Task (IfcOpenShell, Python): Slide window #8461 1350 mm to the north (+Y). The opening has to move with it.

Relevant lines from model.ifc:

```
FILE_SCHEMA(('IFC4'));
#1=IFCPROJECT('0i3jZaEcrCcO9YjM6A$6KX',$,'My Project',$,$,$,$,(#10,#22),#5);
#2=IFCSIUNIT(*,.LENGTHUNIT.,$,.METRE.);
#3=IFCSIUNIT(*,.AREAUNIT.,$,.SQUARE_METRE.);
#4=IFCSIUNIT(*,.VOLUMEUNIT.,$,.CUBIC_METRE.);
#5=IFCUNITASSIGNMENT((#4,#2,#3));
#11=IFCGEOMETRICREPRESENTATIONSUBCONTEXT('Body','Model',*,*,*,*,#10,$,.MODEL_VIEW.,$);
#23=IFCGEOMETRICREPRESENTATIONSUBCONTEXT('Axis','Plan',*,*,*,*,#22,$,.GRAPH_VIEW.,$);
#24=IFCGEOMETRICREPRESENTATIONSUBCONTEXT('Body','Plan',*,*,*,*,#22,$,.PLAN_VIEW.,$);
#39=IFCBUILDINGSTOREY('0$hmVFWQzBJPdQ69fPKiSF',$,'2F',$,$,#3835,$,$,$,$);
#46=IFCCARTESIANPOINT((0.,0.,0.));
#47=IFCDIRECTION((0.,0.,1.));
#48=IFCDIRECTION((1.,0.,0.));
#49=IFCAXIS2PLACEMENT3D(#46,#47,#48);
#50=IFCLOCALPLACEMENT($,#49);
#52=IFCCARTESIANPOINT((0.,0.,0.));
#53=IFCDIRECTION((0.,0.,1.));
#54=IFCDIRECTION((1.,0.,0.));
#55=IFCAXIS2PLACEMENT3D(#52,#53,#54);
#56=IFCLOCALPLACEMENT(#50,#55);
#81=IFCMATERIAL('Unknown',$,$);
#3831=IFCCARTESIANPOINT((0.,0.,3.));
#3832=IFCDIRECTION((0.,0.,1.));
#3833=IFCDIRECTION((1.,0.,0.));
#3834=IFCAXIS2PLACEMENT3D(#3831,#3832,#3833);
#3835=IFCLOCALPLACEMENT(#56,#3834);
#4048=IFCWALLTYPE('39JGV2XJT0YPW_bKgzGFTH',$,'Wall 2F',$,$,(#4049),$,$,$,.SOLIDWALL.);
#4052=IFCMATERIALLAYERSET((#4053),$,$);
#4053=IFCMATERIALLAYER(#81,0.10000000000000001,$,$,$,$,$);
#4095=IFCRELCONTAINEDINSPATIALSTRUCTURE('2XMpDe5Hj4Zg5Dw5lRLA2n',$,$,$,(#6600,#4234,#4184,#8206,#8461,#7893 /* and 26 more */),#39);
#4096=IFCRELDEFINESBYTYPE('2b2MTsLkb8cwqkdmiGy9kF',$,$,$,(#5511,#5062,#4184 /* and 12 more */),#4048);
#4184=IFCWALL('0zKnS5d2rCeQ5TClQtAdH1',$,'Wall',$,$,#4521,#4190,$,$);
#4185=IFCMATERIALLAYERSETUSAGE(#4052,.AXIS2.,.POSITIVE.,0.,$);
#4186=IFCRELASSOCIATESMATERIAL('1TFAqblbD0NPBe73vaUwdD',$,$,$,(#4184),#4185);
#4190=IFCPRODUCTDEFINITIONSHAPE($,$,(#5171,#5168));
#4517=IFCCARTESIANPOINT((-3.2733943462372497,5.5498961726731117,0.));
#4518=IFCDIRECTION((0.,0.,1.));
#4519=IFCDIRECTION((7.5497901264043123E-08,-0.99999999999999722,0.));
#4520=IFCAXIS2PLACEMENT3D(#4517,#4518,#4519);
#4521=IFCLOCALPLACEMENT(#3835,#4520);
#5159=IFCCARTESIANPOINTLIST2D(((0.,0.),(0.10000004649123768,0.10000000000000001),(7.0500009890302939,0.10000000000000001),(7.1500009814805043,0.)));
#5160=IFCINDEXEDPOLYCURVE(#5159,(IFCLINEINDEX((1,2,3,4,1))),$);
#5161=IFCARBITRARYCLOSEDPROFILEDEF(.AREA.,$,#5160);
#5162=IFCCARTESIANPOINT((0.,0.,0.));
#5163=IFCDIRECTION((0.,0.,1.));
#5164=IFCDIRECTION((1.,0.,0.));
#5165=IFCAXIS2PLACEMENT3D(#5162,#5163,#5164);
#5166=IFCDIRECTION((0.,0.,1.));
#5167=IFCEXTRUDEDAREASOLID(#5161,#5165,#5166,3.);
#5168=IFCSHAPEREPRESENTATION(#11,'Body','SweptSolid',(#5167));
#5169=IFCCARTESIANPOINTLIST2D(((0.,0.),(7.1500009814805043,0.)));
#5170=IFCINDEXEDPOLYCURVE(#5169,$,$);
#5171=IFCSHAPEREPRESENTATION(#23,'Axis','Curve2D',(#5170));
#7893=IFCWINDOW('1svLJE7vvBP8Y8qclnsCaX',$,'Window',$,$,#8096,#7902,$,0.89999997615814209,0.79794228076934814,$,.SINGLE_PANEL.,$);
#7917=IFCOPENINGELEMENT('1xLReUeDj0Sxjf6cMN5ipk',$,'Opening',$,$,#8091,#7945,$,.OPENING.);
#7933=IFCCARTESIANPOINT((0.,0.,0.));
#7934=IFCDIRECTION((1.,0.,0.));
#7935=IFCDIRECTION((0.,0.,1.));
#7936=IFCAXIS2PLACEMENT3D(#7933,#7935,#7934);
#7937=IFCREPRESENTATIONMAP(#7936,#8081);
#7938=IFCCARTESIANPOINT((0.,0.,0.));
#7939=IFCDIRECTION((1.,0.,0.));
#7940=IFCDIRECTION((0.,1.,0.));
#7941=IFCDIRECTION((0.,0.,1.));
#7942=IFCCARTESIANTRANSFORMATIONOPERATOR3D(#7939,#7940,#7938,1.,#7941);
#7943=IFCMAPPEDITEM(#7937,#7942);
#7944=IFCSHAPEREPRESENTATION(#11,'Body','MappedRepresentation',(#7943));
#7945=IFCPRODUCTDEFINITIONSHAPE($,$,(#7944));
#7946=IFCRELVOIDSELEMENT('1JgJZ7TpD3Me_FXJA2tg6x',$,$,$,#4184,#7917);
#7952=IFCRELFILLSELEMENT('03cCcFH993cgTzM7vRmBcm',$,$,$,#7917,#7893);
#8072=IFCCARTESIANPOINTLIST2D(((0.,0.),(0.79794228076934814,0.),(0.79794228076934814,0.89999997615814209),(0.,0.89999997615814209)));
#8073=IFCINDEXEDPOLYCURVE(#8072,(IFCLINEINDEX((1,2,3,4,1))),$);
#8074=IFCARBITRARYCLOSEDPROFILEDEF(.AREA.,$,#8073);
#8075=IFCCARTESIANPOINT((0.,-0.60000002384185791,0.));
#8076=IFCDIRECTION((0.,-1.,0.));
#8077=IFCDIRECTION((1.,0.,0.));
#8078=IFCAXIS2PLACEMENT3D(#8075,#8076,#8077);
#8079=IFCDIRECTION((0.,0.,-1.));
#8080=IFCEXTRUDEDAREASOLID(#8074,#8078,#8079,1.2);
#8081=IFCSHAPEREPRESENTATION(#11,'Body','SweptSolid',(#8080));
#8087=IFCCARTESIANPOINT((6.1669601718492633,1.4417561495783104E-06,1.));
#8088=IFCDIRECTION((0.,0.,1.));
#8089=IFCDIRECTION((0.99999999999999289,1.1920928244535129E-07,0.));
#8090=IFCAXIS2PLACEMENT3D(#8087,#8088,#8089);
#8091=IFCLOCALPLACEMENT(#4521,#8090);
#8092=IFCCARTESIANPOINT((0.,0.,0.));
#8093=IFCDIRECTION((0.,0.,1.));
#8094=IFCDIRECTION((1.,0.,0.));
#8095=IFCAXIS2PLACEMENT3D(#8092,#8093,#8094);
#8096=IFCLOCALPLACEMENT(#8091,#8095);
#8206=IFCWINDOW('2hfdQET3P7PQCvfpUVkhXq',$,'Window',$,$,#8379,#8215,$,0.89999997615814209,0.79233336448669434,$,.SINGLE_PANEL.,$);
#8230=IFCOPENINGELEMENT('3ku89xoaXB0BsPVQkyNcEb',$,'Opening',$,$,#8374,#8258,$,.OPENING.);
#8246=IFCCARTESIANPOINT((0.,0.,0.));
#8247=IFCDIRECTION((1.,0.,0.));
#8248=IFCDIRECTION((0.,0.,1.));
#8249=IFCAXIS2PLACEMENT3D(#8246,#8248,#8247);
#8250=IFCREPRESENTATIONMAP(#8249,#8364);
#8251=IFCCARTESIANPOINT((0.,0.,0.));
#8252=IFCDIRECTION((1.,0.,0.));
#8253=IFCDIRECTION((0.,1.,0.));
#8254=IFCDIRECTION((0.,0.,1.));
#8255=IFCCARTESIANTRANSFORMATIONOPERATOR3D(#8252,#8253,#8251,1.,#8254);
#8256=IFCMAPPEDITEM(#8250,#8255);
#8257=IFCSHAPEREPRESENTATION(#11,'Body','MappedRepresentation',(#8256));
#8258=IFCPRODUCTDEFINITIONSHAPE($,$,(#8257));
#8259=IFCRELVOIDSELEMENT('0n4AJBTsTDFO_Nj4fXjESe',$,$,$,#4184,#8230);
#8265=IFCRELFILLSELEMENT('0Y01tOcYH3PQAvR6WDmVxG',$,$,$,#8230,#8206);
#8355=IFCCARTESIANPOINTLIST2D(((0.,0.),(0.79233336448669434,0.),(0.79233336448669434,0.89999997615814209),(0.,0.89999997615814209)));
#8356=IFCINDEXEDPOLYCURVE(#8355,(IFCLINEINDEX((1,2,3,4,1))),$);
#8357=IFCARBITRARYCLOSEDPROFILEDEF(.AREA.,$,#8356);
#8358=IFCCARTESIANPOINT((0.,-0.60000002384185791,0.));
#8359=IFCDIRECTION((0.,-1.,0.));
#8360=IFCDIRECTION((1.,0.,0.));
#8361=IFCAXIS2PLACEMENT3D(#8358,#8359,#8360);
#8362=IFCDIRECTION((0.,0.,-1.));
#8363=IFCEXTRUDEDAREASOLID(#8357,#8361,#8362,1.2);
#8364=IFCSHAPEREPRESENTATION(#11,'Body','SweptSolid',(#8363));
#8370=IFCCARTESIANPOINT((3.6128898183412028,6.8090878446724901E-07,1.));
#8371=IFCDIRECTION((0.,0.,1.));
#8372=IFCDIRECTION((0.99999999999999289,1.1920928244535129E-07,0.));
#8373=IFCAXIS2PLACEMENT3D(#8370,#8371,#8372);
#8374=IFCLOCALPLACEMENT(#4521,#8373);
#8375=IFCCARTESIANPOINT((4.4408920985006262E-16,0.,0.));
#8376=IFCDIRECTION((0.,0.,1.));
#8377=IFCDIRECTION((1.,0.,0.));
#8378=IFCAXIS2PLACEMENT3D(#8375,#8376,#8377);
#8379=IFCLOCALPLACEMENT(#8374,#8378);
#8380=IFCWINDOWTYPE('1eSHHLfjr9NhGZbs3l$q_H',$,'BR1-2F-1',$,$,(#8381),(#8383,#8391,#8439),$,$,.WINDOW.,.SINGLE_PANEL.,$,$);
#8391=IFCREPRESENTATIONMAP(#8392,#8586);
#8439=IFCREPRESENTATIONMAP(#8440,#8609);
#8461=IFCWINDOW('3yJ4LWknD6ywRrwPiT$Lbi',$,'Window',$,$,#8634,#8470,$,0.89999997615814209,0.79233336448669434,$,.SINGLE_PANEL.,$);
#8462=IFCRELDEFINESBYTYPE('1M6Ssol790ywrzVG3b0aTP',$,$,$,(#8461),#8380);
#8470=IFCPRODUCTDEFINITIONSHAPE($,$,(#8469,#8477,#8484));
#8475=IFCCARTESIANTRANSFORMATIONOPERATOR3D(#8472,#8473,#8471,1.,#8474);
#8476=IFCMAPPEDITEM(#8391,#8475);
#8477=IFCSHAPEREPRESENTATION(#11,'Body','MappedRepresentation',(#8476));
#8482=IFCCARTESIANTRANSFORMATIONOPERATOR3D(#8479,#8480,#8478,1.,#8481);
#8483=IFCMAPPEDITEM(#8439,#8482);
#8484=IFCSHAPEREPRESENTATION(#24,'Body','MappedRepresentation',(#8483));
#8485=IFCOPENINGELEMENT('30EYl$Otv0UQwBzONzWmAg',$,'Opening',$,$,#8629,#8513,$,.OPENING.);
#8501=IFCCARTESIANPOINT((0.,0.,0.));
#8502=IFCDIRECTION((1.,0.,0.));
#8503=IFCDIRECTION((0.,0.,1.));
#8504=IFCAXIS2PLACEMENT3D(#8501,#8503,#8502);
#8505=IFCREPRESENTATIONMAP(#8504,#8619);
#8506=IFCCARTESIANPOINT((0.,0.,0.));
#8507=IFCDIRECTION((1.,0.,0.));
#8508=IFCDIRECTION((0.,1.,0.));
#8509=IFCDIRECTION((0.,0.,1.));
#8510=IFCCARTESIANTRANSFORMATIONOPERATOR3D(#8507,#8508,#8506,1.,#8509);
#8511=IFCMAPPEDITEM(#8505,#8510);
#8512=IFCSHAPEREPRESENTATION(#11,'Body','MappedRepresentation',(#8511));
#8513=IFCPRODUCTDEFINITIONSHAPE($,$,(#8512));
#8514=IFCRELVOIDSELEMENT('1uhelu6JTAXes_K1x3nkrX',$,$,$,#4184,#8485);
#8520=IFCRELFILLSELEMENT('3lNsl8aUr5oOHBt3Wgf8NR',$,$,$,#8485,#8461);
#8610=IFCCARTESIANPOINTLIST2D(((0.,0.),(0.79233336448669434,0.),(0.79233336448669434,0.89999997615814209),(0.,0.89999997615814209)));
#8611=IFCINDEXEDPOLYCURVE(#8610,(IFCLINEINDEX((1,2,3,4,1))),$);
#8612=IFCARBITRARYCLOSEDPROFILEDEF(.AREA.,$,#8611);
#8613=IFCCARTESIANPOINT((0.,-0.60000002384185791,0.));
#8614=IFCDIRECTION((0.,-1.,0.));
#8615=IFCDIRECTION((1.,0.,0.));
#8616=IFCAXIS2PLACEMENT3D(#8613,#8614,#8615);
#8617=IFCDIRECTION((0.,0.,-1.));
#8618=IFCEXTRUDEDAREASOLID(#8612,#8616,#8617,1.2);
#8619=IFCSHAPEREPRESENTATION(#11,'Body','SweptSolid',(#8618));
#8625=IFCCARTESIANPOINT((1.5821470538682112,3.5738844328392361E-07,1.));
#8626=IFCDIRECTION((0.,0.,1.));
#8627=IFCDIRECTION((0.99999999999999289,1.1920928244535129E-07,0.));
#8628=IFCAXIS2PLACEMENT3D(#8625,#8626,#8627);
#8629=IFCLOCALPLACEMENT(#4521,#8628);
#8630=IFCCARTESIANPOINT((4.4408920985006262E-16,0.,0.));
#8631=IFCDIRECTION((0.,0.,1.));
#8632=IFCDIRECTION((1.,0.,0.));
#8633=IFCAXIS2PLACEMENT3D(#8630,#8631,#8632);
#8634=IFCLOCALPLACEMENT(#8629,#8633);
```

```python
import ifcopenshell
import ifcopenshell.api.geometry
import ifcopenshell.util.placement

model = ifcopenshell.open("model.ifc")

window = model.by_guid("3yJ4LWknD6ywRrwPiT$Lbi")
opening = window.FillsVoids[0].RelatingOpeningElement
wall = opening.VoidsElements[0].RelatingBuildingElement

wall_matrix = ifcopenshell.util.placement.get_local_placement(wall.ObjectPlacement)
shift = wall_matrix[:3, 0] * -1.35
before = ifcopenshell.util.placement.get_local_placement(window.ObjectPlacement)[:3, 3].copy()

# The window is placed relative to its opening, so it follows when the opening moves.
matrix = ifcopenshell.util.placement.get_local_placement(opening.ObjectPlacement)
matrix[:3, 3] += shift
ifcopenshell.api.geometry.edit_object_placement(
    model, product=opening, matrix=matrix, is_si=False, should_transform_children=True
)

after = ifcopenshell.util.placement.get_local_placement(window.ObjectPlacement)[:3, 3]
print("window moved by", (after - before).round(3) + 0.0)

model.write("model_updated.ifc")
```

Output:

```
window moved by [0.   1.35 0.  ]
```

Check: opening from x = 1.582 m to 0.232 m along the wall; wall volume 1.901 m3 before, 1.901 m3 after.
